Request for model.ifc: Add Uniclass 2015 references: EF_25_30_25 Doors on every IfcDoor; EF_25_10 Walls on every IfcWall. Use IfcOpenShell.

First a look at what the model holds.

```python
import ifcopenshell

model = ifcopenshell.open("model.ifc")
print(model.schema)
print("classifications:", [c.Name for c in model.by_type("IfcClassification")])
for ifc_class in ("IfcDoor", "IfcRoof", "IfcStair", "IfcWall", "IfcWindow"):
    print(ifc_class, len(model.by_type(ifc_class)))
```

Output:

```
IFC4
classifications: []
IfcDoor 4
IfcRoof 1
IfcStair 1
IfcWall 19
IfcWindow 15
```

```python
import ifcopenshell
import ifcopenshell.api.classification

model = ifcopenshell.open("model.ifc")

system = ifcopenshell.api.classification.add_classification(model, classification="Uniclass 2015")

codes = {
    "IfcDoor": ("EF_25_30_25", "Doors"),
    "IfcWall": ("EF_25_10", "Walls"),
}
for ifc_class, (code, name) in codes.items():
    products = model.by_type(ifc_class)
    ifcopenshell.api.classification.add_reference(
        model, products=products, classification=system, identification=code, name=name
    )
    print(code, len(products))

model.write("model-out.ifc")
```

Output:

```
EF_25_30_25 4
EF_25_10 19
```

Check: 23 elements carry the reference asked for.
